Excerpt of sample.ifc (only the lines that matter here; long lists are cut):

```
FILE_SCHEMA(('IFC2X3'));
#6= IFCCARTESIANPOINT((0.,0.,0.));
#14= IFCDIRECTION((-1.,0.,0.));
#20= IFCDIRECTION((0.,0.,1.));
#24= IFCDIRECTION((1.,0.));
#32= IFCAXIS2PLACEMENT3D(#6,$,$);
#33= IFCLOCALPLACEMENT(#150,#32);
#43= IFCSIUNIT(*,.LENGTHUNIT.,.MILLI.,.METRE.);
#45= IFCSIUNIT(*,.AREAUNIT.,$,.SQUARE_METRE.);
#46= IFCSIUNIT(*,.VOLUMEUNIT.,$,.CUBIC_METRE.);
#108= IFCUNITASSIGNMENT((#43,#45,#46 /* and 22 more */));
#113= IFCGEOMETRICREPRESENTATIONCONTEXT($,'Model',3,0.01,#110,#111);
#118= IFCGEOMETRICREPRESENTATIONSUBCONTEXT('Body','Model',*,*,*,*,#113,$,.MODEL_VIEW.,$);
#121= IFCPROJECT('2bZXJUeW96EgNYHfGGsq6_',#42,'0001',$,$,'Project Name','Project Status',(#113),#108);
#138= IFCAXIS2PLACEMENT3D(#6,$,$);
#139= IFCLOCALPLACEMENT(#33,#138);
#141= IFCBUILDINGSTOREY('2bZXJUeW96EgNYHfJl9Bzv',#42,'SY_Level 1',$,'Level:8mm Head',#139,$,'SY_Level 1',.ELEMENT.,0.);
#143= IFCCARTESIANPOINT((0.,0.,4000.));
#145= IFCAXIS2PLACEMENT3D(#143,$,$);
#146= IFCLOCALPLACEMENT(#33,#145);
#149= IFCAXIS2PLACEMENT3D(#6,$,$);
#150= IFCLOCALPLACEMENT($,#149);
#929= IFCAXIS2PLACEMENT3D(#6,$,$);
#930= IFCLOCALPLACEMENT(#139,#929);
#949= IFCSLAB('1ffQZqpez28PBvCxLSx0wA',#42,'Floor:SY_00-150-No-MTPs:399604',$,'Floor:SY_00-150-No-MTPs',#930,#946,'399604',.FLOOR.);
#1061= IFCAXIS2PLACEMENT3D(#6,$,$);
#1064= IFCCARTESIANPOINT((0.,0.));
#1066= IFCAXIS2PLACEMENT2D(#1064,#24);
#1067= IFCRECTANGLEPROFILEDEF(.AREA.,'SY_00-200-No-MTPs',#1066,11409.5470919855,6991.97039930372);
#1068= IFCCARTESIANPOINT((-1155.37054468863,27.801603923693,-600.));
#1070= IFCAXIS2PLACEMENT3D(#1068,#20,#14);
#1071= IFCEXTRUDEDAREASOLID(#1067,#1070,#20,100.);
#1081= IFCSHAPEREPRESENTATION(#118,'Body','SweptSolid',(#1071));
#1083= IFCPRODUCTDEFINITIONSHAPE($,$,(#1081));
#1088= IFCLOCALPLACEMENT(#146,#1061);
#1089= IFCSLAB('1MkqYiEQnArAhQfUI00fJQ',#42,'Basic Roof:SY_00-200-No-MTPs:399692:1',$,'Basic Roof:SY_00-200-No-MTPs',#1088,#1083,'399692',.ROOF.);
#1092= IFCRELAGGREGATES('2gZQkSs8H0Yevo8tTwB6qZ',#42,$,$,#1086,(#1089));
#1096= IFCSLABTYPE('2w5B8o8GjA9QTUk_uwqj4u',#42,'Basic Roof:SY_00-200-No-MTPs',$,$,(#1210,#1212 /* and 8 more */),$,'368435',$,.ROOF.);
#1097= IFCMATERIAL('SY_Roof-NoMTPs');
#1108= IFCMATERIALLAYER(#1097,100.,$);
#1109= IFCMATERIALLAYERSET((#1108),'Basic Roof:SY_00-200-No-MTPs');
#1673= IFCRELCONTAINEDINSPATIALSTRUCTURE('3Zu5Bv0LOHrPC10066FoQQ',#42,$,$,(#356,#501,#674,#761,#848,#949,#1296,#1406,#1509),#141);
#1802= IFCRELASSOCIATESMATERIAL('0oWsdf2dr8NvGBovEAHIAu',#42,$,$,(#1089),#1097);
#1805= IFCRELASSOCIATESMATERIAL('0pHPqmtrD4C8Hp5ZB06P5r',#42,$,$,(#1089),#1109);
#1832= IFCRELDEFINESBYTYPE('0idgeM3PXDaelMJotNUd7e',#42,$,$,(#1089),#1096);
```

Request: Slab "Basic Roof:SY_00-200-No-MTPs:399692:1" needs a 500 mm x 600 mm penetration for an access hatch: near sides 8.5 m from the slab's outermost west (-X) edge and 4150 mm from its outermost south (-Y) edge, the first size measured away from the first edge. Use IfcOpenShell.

```python
import numpy as np
import ifcopenshell
import ifcopenshell.api.feature
import ifcopenshell.api.geometry
import ifcopenshell.api.root
import ifcopenshell.geom
import ifcopenshell.util.placement
import ifcopenshell.util.representation
import ifcopenshell.util.shape
import ifcopenshell.util.unit

model = ifcopenshell.open("sample.ifc")
unit_scale = ifcopenshell.util.unit.calculate_unit_scale(model)
settings = ifcopenshell.geom.settings()


def volume(element):
    """Net volume in cubic metres, openings subtracted."""
    shape = ifcopenshell.geom.create_shape(settings, element)
    return ifcopenshell.util.shape.get_volume(shape.geometry)


slab = model.by_guid("1MkqYiEQnArAhQfUI00fJQ")
before = volume(slab)

# Extent in the slab's own axes, in metres. The edges named are its -X and -Y sides.
slab_shape = ifcopenshell.geom.create_shape(settings, slab)
vertices = ifcopenshell.util.shape.get_vertices(slab_shape.geometry)
x_min, y_min, bottom = vertices.min(axis=0)
top = vertices[:, 2].max()

opening = ifcopenshell.api.root.create_entity(model, ifc_class="IfcOpeningElement", name="Access hatch opening")
context = ifcopenshell.util.representation.get_context(model, "Model", "Body", "MODEL_VIEW")
width, depth = 0.5, 0.6
outline = [(0.0, 0.0), (width, 0.0), (width, depth), (0.0, depth), (0.0, 0.0)]
# Overshoot both faces by 50 mm so the cut is clean.
shape = ifcopenshell.api.geometry.add_slab_representation(
    model, context=context, depth=top - bottom + 0.1, polyline=outline
)
ifcopenshell.api.geometry.assign_representation(model, product=opening, representation=shape)

matrix = ifcopenshell.util.placement.get_local_placement(slab.ObjectPlacement)
matrix[:, 3] = matrix @ np.append(np.array([x_min + 8.5, y_min + 4.15, bottom - 0.05]) / unit_scale, 1.0)
ifcopenshell.api.geometry.edit_object_placement(model, product=opening, matrix=matrix, is_si=False)
ifcopenshell.api.feature.add_feature(model, feature=opening, element=slab)

after = volume(slab)

print(f"slab volume {before:.3f} -> {after:.3f} m3")

model.write("sample_edited.ifc")
```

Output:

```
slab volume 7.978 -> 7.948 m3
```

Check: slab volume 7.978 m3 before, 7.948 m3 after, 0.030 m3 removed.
